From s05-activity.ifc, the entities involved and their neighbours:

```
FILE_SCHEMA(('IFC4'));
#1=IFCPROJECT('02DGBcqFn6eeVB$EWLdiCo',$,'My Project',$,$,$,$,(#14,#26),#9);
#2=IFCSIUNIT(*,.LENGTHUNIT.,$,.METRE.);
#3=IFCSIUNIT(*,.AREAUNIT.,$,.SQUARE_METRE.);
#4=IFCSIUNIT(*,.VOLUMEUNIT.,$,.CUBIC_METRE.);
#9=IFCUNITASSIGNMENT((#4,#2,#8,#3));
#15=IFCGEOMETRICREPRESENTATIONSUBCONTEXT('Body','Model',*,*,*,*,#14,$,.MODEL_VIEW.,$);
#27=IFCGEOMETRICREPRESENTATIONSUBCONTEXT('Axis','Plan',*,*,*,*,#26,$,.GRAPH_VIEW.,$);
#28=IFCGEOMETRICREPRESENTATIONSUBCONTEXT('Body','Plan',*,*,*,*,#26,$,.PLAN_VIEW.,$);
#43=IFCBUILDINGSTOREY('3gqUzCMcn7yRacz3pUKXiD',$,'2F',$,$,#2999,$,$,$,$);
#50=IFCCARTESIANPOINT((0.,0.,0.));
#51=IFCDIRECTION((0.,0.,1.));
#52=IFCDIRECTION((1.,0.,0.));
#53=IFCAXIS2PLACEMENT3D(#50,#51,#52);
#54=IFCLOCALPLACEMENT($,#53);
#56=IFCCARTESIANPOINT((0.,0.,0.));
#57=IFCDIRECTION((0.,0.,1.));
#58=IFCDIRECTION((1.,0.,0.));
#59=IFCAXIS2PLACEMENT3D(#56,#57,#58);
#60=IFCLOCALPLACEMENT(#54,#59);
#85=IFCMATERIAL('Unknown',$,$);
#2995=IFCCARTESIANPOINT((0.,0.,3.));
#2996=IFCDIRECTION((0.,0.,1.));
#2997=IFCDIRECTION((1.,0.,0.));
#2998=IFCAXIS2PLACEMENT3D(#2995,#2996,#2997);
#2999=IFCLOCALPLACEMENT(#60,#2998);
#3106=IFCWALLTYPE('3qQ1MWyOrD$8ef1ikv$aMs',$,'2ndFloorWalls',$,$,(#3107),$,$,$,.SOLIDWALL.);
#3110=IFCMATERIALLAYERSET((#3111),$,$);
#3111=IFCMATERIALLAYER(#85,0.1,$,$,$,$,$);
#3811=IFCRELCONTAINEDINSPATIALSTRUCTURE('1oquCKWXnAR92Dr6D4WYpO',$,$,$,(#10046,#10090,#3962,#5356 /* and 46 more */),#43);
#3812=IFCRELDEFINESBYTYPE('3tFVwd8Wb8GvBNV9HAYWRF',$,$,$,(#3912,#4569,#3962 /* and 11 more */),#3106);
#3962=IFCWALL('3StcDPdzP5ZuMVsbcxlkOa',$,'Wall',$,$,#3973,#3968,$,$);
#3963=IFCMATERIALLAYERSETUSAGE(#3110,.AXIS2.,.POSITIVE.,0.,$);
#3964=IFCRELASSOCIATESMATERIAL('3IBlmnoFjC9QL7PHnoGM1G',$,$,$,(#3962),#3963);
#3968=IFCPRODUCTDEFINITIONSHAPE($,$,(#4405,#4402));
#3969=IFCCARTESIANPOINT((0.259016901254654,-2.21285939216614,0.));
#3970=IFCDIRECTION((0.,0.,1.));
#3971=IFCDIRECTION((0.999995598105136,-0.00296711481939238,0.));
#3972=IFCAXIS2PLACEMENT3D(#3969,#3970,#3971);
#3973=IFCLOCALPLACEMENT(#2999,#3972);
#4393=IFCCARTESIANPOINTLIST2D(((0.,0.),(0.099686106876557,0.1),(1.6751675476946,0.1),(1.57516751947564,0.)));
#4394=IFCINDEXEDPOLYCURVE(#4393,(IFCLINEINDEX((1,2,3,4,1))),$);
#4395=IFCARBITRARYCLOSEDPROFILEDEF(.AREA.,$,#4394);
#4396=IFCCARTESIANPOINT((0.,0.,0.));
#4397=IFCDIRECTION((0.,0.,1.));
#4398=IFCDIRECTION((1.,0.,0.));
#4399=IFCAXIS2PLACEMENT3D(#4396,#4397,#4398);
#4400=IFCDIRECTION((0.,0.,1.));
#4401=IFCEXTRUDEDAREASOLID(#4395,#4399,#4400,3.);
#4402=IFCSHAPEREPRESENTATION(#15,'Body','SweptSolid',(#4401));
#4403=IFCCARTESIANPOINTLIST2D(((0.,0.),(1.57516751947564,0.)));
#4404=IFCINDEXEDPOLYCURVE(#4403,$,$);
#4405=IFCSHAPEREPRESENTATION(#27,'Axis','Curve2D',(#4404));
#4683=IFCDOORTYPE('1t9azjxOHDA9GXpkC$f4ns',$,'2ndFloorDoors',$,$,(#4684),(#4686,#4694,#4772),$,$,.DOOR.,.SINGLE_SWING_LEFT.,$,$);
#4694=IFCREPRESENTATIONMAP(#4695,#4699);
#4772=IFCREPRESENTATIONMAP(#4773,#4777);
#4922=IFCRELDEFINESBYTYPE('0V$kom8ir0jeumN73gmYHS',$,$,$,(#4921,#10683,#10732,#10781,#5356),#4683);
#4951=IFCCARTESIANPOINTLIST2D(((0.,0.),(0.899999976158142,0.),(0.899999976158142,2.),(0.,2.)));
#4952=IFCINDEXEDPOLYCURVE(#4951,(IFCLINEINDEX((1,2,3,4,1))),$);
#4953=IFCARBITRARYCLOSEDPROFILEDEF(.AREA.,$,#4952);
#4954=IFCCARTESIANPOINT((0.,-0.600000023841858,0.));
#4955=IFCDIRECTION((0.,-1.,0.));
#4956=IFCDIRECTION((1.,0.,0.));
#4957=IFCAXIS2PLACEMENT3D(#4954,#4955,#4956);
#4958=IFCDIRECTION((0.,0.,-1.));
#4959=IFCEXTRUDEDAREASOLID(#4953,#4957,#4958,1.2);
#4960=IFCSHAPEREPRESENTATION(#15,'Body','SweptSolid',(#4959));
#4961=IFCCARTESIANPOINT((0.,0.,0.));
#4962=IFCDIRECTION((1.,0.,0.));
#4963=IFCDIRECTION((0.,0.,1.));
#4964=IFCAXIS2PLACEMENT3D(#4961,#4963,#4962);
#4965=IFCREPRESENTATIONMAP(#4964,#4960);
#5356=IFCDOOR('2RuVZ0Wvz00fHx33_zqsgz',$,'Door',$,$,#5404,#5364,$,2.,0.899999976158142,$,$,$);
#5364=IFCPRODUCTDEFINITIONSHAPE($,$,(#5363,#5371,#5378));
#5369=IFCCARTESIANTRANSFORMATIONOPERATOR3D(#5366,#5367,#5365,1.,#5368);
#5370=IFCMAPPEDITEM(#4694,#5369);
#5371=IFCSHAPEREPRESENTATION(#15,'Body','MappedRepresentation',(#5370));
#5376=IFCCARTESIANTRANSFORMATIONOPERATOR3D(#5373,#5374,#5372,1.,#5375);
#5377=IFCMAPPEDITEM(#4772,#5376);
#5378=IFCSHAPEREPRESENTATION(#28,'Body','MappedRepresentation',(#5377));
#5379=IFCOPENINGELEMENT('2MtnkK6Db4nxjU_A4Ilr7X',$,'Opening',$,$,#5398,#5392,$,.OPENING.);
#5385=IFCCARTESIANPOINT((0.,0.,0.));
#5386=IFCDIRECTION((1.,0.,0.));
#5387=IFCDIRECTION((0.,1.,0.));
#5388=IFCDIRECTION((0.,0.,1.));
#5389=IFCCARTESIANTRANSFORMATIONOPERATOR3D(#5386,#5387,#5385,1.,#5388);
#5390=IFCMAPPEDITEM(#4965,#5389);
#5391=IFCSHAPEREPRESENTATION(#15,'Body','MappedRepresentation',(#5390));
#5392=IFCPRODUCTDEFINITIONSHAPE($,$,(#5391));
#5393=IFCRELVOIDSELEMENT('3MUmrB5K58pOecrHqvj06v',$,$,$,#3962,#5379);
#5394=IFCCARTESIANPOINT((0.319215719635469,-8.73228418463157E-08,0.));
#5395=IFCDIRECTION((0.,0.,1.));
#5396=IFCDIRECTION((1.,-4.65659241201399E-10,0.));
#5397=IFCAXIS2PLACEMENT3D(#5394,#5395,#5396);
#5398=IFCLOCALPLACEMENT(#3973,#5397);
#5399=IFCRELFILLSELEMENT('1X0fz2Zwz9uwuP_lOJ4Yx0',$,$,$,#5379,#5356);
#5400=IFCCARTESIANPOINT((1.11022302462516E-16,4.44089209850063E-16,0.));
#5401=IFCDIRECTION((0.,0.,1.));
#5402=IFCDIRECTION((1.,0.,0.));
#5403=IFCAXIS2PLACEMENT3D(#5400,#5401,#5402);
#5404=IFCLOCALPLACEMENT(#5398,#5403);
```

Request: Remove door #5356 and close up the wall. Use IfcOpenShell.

```python
import ifcopenshell
import ifcopenshell.api.feature
import ifcopenshell.api.root
import ifcopenshell.geom
import ifcopenshell.util.shape

model = ifcopenshell.open("s05-activity.ifc")
settings = ifcopenshell.geom.settings()


def volume(element):
    """Net volume in cubic metres, openings subtracted."""
    shape = ifcopenshell.geom.create_shape(settings, element)
    return ifcopenshell.util.shape.get_volume(shape.geometry)


door = model.by_guid("2RuVZ0Wvz00fHx33_zqsgz")
opening = door.FillsVoids[0].RelatingOpeningElement
wall = opening.VoidsElements[0].RelatingBuildingElement
before = volume(wall)

ifcopenshell.api.root.remove_product(model, product=door)
ifcopenshell.api.feature.remove_feature(model, feature=opening)

after = volume(wall)

print(f"wall volume {before:.3f} -> {after:.3f} m3")

model.write("s05-activity_edited.ifc")
```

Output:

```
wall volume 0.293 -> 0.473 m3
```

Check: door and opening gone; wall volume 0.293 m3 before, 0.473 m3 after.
